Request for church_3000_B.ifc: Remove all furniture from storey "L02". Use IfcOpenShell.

First a look at what the model holds.

```python
import ifcopenshell
import ifcopenshell.util.element

model = ifcopenshell.open("church_3000_B.ifc")
print(model.schema)
storey = next(s for s in model.by_type("IfcBuildingStorey") if s.Name == "L02")
furniture = [e for e in ifcopenshell.util.element.get_decomposition(storey) if e.is_a("IfcFurnishingElement")]
seen = {}
for e in furniture:
    element_type = ifcopenshell.util.element.get_type(e)
    name = element_type.Name if element_type not in (None, e) else None
    seen[name] = seen.get(name, 0) + 1
for name, count in sorted(seen.items(), key=str):
    print(count, "x", name)
```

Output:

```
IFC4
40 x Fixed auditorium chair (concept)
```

```python
import ifcopenshell
import ifcopenshell.api.root
import ifcopenshell.util.element

model = ifcopenshell.open("church_3000_B.ifc")

storey = next(s for s in model.by_type("IfcBuildingStorey") if s.Name == "L02")
furniture = [e for e in ifcopenshell.util.element.get_decomposition(storey) if e.is_a("IfcFurnishingElement")]

for e in furniture:
    ifcopenshell.api.root.remove_product(model, product=e)
print(len(furniture), "removed")

model.write("church_3000_B-out.ifc")
```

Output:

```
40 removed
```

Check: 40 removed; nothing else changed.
